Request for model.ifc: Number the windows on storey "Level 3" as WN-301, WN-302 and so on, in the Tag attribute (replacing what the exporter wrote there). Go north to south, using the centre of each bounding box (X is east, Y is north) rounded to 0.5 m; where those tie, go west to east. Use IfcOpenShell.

First a look at what the model holds.

```python
import ifcopenshell
import ifcopenshell.util.element
import ifcopenshell.util.placement

model = ifcopenshell.open("model.ifc")
print(model.schema)
storey = next(s for s in model.by_type("IfcBuildingStorey") if s.Name == "Level 3")
windows = [e for e in ifcopenshell.util.element.get_decomposition(storey) if e.is_a("IfcWindow")]
for e in sorted(windows, key=lambda e: e.id()):
    origin = ifcopenshell.util.placement.get_local_placement(e.ObjectPlacement)[:3, 3]
    print(e.id(), e.Tag, e.Name, origin.round(2) + 0.0, sep=" | ")
```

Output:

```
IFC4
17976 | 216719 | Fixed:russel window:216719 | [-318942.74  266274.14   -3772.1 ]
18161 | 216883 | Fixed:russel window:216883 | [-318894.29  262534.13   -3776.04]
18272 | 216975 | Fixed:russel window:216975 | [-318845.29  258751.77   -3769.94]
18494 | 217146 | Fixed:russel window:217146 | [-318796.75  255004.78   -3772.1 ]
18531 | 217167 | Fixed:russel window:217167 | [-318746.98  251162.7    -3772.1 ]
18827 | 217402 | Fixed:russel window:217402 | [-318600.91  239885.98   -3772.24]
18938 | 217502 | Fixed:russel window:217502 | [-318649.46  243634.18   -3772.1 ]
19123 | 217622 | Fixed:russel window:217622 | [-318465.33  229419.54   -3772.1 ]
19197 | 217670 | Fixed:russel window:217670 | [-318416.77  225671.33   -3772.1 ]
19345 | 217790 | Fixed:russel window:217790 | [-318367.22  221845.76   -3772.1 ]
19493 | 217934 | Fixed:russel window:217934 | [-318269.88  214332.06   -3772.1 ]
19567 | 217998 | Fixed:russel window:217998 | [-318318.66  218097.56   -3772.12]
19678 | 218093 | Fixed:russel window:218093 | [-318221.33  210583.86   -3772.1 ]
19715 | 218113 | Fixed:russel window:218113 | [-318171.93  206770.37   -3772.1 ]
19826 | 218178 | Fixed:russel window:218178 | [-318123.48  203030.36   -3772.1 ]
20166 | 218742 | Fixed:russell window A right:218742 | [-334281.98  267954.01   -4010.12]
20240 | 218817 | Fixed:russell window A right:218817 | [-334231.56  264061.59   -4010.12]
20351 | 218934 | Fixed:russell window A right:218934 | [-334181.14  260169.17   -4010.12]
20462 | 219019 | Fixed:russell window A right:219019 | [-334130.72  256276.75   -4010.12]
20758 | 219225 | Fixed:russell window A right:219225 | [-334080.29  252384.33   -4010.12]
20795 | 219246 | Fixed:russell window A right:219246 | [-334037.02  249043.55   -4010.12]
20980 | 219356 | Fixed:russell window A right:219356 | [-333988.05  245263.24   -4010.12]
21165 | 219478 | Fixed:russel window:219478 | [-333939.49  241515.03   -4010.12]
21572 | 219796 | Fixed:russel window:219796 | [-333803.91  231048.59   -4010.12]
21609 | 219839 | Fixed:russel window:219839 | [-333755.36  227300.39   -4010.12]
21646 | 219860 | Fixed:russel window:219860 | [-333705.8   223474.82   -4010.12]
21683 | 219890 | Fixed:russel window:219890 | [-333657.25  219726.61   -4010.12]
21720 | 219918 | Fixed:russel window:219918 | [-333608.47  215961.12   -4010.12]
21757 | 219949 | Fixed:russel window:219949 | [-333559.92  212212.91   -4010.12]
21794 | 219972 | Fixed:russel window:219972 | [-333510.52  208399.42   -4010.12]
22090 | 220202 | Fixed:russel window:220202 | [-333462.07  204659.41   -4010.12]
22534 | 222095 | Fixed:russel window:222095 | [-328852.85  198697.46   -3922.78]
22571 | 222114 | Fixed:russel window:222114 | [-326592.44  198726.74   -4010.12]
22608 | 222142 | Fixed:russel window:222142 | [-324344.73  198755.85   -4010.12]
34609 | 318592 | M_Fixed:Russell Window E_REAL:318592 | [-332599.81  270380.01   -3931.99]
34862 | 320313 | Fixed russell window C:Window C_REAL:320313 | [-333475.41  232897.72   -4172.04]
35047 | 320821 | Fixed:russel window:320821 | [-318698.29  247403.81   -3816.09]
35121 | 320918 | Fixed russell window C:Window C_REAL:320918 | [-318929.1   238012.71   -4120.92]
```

```python
import ifcopenshell
import ifcopenshell.geom
import ifcopenshell.util.element
import ifcopenshell.util.shape

model = ifcopenshell.open("model.ifc")
settings = ifcopenshell.geom.settings()
settings.set("use-world-coords", True)


def centre(element):
    shape = ifcopenshell.geom.create_shape(settings, element)
    return ifcopenshell.util.shape.get_bbox_centroid(shape.geometry)


storey = next(s for s in model.by_type("IfcBuildingStorey") if s.Name == "Level 3")
windows = [e for e in ifcopenshell.util.element.get_decomposition(storey) if e.is_a("IfcWindow")]

# Insertion points can sit at a corner or the storey origin, so sort by the geometry (in metres).
centres = {e: centre(e) for e in windows}
windows.sort(key=lambda e: (-round(centres[e][1] / 0.5), centres[e][0]))

for i, e in enumerate(windows, start=1):
    number = f"WN-3{i:02d}"
    e.Tag = number
    print(e.id(), number)

model.write("model_v2.ifc")
```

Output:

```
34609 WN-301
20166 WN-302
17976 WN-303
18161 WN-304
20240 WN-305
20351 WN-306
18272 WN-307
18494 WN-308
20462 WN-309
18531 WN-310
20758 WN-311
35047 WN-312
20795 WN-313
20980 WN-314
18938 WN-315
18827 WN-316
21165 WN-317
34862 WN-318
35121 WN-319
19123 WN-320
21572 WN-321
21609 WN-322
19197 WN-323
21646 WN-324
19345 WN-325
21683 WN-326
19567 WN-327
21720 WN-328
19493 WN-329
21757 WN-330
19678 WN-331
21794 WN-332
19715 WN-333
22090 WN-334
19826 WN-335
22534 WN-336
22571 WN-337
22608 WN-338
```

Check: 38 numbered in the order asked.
